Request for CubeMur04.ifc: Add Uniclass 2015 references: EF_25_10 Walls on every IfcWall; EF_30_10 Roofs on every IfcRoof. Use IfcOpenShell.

First a look at what the model holds.

```python
import ifcopenshell

model = ifcopenshell.open("CubeMur04.ifc")
print(model.schema)
print("classifications:", [c.Name for c in model.by_type("IfcClassification")])
for ifc_class in ("IfcDoor", "IfcRoof", "IfcStair", "IfcWall", "IfcWindow"):
    print(ifc_class, len(model.by_type(ifc_class)))
```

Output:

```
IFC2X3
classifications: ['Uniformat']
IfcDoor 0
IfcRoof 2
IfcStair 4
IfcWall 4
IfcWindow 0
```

```python
import ifcopenshell
import ifcopenshell.api.classification

model = ifcopenshell.open("CubeMur04.ifc")

# IFC2X3 requires Source and Edition and has no link from the project to the system.
system = model.create_entity("IfcClassification", Source="NBS", Edition="2015", Name="Uniclass 2015")

codes = {
    "IfcWall": ("EF_25_10", "Walls"),
    "IfcRoof": ("EF_30_10", "Roofs"),
}
for ifc_class, (code, name) in codes.items():
    products = model.by_type(ifc_class)
    ifcopenshell.api.classification.add_reference(
        model, products=products, classification=system, identification=code, name=name
    )
    print(code, len(products))

model.write("CubeMur04_rev.ifc")
```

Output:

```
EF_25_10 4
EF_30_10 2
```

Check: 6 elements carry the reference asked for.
